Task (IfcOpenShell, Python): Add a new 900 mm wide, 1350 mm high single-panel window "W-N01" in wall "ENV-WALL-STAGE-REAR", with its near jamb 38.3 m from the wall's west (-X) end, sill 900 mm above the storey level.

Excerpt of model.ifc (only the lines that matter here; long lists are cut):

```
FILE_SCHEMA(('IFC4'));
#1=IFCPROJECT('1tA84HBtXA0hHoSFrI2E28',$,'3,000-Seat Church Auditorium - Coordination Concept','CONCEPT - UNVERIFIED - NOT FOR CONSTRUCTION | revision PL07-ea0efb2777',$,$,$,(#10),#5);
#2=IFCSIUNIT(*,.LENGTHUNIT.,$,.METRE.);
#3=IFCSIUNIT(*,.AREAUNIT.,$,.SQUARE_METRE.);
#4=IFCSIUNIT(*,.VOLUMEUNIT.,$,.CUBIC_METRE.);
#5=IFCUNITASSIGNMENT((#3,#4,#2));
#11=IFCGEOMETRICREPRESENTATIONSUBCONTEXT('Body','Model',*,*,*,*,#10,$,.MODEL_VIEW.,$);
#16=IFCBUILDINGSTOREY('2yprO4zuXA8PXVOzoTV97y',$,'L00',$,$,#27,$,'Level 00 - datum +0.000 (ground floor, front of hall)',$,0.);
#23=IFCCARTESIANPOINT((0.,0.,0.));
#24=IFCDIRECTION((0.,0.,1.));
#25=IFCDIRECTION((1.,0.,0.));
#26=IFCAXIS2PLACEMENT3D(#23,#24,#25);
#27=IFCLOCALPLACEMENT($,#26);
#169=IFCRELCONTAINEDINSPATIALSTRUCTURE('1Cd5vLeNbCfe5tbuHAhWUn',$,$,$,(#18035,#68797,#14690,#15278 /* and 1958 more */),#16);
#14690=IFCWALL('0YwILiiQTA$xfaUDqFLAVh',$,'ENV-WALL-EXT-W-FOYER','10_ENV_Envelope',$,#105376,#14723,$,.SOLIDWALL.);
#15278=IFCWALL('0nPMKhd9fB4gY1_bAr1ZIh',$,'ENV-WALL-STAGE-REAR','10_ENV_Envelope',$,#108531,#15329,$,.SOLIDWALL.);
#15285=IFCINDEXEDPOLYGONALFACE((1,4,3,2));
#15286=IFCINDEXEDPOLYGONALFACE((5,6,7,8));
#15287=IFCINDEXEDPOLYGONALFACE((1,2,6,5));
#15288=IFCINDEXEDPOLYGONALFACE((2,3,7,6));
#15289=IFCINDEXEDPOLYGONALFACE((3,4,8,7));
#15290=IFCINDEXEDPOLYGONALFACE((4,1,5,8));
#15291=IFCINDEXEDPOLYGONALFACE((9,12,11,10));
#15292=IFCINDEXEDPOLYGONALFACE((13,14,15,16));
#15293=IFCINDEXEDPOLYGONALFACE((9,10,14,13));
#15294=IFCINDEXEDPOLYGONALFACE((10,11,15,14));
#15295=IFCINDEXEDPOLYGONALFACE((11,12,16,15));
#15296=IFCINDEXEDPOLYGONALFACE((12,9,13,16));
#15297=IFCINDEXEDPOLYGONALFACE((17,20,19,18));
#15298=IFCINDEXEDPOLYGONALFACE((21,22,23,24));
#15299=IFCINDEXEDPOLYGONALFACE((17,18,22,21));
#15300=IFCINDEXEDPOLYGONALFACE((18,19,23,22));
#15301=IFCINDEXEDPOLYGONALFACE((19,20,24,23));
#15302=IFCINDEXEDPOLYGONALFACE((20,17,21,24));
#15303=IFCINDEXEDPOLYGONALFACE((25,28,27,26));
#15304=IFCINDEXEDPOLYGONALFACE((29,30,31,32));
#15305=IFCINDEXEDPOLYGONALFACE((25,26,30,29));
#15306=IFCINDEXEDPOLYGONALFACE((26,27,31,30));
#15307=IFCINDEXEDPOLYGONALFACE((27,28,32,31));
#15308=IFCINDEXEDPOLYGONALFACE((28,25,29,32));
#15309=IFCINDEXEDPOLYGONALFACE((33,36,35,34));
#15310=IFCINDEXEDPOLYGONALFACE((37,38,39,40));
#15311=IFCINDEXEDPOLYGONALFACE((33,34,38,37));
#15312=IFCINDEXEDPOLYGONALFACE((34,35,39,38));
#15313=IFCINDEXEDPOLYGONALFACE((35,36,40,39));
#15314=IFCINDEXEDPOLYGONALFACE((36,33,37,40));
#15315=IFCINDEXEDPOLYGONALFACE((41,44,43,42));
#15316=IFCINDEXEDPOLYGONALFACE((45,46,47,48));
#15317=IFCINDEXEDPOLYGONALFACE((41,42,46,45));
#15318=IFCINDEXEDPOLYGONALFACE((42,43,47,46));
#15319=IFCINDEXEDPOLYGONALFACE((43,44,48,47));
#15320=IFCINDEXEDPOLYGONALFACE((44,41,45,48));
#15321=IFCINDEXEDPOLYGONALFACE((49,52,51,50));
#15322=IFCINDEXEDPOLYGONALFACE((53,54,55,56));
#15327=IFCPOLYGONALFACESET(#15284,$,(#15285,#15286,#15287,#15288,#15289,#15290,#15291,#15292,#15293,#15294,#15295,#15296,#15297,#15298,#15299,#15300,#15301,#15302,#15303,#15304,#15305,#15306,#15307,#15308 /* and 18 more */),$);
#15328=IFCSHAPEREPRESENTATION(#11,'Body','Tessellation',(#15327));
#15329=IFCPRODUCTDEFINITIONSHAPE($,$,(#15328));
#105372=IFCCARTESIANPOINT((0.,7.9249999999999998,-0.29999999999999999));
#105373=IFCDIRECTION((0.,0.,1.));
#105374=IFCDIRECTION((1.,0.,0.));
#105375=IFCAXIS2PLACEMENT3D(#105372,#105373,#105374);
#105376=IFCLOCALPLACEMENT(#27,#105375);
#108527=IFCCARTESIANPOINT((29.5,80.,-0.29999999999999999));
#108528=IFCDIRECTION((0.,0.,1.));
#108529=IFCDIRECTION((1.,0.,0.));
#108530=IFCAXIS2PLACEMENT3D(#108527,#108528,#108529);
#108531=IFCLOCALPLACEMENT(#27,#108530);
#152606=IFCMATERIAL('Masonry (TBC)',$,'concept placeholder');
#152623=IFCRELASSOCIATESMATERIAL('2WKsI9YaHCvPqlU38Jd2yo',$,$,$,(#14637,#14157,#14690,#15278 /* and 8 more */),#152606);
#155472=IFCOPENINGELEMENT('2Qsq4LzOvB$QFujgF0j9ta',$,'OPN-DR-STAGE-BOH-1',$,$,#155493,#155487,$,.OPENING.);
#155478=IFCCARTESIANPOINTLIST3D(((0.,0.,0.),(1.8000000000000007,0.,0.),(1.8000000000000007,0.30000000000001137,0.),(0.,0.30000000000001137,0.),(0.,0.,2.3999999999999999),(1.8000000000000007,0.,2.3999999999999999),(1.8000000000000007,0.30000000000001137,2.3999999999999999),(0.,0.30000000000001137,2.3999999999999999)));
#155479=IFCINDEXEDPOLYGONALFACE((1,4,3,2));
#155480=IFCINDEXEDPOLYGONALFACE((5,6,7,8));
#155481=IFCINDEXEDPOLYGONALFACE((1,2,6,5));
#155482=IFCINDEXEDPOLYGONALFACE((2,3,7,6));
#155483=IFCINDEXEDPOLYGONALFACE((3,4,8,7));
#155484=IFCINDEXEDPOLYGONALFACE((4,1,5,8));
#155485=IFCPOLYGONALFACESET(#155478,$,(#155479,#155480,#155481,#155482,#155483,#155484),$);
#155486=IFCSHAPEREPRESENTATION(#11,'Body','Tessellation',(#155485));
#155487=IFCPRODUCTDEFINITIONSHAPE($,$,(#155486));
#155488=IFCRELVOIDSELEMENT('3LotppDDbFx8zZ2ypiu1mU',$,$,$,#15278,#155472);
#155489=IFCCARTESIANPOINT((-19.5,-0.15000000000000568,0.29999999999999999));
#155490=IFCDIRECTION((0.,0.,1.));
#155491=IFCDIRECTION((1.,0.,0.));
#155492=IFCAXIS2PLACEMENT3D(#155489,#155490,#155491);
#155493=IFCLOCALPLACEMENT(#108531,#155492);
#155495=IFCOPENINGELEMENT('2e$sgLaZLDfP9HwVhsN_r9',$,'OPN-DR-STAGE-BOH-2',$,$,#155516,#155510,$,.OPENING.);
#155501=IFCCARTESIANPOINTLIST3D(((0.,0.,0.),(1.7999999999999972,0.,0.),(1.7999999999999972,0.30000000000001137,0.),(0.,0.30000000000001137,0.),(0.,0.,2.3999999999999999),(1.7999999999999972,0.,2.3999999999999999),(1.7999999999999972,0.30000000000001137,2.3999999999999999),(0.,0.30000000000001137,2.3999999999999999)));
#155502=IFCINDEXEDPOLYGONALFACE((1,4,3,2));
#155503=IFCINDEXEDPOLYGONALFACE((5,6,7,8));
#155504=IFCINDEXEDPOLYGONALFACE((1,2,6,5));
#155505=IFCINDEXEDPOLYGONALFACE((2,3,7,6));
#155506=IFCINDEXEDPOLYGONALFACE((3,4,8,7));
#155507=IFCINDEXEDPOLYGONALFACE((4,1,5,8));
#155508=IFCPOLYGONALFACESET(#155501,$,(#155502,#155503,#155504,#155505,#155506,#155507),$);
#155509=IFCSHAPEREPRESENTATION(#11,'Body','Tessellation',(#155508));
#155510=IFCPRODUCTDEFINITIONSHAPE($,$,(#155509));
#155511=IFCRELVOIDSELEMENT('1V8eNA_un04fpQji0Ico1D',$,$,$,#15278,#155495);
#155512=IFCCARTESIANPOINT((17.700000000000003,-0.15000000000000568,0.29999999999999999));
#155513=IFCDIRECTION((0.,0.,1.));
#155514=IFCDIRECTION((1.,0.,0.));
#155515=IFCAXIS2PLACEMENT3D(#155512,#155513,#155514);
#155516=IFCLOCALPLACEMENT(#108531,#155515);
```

```python
import numpy as np
import ifcopenshell
import ifcopenshell.api.feature
import ifcopenshell.api.geometry
import ifcopenshell.api.root
import ifcopenshell.api.spatial
import ifcopenshell.geom
import ifcopenshell.util.element
import ifcopenshell.util.placement
import ifcopenshell.util.representation
import ifcopenshell.util.shape
import ifcopenshell.util.unit

model = ifcopenshell.open("model.ifc")
unit_scale = ifcopenshell.util.unit.calculate_unit_scale(model)
settings = ifcopenshell.geom.settings()


def volume(element):
    """Net volume in cubic metres, openings subtracted."""
    shape = ifcopenshell.geom.create_shape(settings, element)
    return ifcopenshell.util.shape.get_volume(shape.geometry)


wall = model.by_guid("0nPMKhd9fB4gY1_bAr1ZIh")
storey = ifcopenshell.util.element.get_container(wall, ifc_class="IfcBuildingStorey")
context = ifcopenshell.util.representation.get_context(model, "Model", "Body", "MODEL_VIEW")
before = volume(wall)

width, height, from_end, sill = 0.9, 1.35, 38.3, 0.9  # metres

# The wall runs along its own X axis, and the end named is its -X end.
wall_shape = ifcopenshell.geom.create_shape(settings, wall)
x, y, z = ifcopenshell.util.shape.get_vertices(wall_shape.geometry).T
start = x.min() + from_end
face, thickness = float(y.min()), float(y.max() - y.min())
wall_matrix = ifcopenshell.util.placement.get_local_placement(wall.ObjectPlacement)
level = ifcopenshell.util.placement.get_local_placement(storey.ObjectPlacement)[2, 3]


def in_wall(x, y):
    """Placement at x, y metres in the wall's axes, at sill height."""
    matrix = wall_matrix.copy()
    matrix[:, 3] = wall_matrix @ np.array([x / unit_scale, y / unit_scale, 0.0, 1.0])
    matrix[2, 3] = level + sill / unit_scale
    return matrix


# Opening: a box that overshoots both wall faces by 50 mm.
opening = ifcopenshell.api.root.create_entity(model, ifc_class="IfcOpeningElement", predefined_type="OPENING")
box = ifcopenshell.api.geometry.add_wall_representation(
    model, context=context, length=width, height=height, thickness=thickness + 0.1
)
ifcopenshell.api.geometry.assign_representation(model, product=opening, representation=box)
ifcopenshell.api.geometry.edit_object_placement(model, product=opening, matrix=in_wall(start, face - 0.05), is_si=False)
ifcopenshell.api.feature.add_feature(model, feature=opening, element=wall)

window = ifcopenshell.api.root.create_entity(model, ifc_class="IfcWindow", name="W-N01", predefined_type="WINDOW")
window.OverallWidth, window.OverallHeight = width / unit_scale, height / unit_scale
window.PartitioningType = "SINGLE_PANEL"
body = ifcopenshell.api.geometry.add_window_representation(
    model,
    context=context,
    overall_width=window.OverallWidth,
    overall_height=window.OverallHeight,
    partition_type="SINGLE_PANEL",
)
ifcopenshell.api.geometry.assign_representation(model, product=window, representation=body)
ifcopenshell.api.spatial.assign_container(model, products=[window], relating_structure=storey)
ifcopenshell.api.feature.add_filling(model, opening=opening, element=window)

# Centre the window in the wall's thickness.
ifcopenshell.api.geometry.edit_object_placement(model, product=window, matrix=in_wall(start, face), is_si=False)
window_shape = ifcopenshell.geom.create_shape(settings, window)
depth = ifcopenshell.util.shape.get_vertices(window_shape.geometry)[:, 1]
offset = face + thickness / 2 - (depth.min() + depth.max()) / 2
ifcopenshell.api.geometry.edit_object_placement(model, product=window, matrix=in_wall(start, offset), is_si=False)

after = volume(wall)

print(f"wall volume {before:.3f} -> {after:.3f} m3")

model.write("model_edited.ifc")
```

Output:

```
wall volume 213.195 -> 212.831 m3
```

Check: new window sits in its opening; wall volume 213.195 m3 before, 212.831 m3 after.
